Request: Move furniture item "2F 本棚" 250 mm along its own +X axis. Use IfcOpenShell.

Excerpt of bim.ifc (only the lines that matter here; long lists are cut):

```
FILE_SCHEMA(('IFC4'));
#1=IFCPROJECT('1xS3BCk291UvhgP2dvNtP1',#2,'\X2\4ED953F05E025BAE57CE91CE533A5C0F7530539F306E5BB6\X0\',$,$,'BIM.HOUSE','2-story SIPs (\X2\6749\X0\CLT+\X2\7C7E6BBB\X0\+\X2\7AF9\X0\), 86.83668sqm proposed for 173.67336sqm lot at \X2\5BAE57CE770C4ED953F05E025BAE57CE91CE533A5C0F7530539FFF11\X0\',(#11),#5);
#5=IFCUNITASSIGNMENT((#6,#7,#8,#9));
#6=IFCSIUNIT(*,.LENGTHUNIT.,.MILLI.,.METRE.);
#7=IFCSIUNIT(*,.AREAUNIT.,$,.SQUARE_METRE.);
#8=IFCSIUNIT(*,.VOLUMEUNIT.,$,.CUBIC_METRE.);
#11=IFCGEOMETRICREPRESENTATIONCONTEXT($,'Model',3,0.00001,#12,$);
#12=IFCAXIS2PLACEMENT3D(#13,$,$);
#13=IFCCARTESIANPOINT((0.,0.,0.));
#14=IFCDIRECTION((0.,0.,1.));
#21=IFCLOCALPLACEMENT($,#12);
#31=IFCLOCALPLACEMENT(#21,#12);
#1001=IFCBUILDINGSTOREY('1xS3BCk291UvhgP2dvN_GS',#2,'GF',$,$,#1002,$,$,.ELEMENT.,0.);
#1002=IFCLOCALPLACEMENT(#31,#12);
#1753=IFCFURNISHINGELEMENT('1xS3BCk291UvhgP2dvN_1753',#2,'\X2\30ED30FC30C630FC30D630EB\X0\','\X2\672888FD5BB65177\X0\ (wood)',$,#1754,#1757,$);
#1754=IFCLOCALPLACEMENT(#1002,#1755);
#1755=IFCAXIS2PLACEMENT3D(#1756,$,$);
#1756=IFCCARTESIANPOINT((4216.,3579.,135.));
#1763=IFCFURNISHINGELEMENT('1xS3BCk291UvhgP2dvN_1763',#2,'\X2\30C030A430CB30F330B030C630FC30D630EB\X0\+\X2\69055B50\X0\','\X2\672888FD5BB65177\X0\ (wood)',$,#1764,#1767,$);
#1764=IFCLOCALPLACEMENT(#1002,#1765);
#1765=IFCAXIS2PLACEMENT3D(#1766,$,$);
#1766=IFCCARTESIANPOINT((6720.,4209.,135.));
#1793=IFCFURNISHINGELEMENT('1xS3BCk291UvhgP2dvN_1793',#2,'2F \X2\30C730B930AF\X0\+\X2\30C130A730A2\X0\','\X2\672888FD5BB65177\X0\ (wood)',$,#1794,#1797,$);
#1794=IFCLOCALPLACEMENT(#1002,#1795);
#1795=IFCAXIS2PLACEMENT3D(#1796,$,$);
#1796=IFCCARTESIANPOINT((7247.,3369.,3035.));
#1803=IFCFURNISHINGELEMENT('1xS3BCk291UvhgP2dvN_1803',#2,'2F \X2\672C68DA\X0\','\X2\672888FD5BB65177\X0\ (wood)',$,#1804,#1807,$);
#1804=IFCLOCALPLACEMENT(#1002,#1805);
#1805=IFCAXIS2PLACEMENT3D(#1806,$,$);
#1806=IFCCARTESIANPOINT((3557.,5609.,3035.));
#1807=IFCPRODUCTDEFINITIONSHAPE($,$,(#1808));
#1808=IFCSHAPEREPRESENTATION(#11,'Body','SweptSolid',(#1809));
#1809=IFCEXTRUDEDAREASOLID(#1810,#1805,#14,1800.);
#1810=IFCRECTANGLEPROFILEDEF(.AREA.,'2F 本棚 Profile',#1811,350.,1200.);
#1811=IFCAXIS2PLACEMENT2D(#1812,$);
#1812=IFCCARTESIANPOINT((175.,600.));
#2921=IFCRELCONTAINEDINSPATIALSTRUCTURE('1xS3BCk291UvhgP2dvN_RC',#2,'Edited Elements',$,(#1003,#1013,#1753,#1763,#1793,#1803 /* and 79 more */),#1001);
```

```python
import ifcopenshell
import ifcopenshell.api.geometry
import ifcopenshell.util.placement
import ifcopenshell.util.unit

model = ifcopenshell.open("bim.ifc")
unit_scale = ifcopenshell.util.unit.calculate_unit_scale(model)

item = model.by_guid("1xS3BCk291UvhgP2dvN_1803")
matrix = ifcopenshell.util.placement.get_local_placement(item.ObjectPlacement)
matrix[:3, 3] += matrix[:3, 0] * 0.25 / unit_scale
ifcopenshell.api.geometry.edit_object_placement(model, product=item, matrix=matrix, is_si=False)

print(ifcopenshell.util.placement.get_local_placement(item.ObjectPlacement).round(3) + 0.0)

model.write("bim_updated.ifc")
```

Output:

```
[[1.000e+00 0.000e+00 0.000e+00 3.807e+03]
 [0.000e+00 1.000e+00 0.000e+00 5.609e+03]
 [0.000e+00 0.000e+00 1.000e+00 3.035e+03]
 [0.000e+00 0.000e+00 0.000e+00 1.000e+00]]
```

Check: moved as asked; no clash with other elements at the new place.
